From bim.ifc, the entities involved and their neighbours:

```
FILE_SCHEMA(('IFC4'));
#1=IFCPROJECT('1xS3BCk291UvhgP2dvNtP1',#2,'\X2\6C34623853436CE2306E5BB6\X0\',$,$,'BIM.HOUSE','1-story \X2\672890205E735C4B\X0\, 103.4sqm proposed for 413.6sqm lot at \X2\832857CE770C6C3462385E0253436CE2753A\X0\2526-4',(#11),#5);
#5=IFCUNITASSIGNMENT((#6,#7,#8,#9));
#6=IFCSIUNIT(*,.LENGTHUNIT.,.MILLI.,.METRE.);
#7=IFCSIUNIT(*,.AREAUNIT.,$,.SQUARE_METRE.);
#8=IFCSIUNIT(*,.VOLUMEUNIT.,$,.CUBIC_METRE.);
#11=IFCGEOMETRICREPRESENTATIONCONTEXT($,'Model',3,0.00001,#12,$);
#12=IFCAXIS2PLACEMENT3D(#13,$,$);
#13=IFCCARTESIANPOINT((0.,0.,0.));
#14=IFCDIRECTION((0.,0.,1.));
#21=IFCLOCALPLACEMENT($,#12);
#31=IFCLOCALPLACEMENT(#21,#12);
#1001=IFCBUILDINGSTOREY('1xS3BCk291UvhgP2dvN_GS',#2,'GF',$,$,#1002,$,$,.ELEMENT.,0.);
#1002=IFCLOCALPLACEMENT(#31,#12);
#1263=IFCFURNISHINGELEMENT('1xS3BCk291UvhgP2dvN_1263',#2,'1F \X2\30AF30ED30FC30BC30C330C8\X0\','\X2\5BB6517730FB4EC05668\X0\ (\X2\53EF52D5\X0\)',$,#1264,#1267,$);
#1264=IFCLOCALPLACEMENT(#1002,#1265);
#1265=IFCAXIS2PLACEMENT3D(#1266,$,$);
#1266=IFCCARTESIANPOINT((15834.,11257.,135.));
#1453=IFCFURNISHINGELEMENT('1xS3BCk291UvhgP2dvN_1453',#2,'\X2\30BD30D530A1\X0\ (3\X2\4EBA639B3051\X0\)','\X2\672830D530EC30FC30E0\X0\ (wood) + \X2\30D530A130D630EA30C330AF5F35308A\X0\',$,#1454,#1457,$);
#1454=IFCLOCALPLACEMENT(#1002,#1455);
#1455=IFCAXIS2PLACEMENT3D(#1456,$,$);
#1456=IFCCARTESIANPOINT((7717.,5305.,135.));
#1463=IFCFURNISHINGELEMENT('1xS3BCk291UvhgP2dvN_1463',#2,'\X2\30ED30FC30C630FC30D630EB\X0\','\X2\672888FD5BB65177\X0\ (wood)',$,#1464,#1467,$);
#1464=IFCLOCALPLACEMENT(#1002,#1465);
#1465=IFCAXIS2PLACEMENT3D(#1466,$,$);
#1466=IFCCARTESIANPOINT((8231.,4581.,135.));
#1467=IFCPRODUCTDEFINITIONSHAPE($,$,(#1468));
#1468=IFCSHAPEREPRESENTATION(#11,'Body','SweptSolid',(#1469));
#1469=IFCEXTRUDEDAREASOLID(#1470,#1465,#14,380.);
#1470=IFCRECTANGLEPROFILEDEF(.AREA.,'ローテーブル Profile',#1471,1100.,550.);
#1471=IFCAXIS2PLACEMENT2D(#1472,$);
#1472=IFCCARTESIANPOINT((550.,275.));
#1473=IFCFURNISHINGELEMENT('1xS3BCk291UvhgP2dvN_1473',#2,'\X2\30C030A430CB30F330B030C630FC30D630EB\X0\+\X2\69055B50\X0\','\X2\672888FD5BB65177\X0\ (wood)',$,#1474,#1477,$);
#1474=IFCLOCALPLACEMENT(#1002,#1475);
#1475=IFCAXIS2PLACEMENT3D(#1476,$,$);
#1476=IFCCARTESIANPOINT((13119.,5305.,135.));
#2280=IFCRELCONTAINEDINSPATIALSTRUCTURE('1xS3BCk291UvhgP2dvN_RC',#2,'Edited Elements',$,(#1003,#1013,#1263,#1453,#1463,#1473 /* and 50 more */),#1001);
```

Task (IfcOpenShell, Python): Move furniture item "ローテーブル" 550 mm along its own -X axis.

```python
import ifcopenshell
import ifcopenshell.api.geometry
import ifcopenshell.util.placement
import ifcopenshell.util.unit

model = ifcopenshell.open("bim.ifc")
unit_scale = ifcopenshell.util.unit.calculate_unit_scale(model)

item = model.by_id(1463)
matrix = ifcopenshell.util.placement.get_local_placement(item.ObjectPlacement)
matrix[:3, 3] -= matrix[:3, 0] * 0.55 / unit_scale
ifcopenshell.api.geometry.edit_object_placement(model, product=item, matrix=matrix, is_si=False)

print(ifcopenshell.util.placement.get_local_placement(item.ObjectPlacement).round(3) + 0.0)

model.write("bim_rev.ifc")
```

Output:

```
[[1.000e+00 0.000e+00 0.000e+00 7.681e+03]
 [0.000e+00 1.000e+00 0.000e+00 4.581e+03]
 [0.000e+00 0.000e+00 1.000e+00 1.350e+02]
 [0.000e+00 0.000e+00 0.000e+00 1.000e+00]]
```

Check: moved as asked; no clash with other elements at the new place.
